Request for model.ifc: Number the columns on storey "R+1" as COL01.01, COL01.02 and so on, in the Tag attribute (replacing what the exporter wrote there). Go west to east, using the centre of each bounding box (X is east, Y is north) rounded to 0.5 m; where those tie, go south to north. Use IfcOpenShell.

First a look at what the model holds.

```python
import ifcopenshell
import ifcopenshell.util.element
import ifcopenshell.util.placement

model = ifcopenshell.open("model.ifc")
print(model.schema)
storey = next(s for s in model.by_type("IfcBuildingStorey") if s.Name == "R+1")
columns = [e for e in ifcopenshell.util.element.get_decomposition(storey) if e.is_a("IfcColumn")]
for e in sorted(columns, key=lambda e: e.id()):
    origin = ifcopenshell.util.placement.get_local_placement(e.ObjectPlacement)[:3, 3]
    print(e.id(), e.Tag, e.Name, origin.round(2) + 0.0, sep=" | ")
```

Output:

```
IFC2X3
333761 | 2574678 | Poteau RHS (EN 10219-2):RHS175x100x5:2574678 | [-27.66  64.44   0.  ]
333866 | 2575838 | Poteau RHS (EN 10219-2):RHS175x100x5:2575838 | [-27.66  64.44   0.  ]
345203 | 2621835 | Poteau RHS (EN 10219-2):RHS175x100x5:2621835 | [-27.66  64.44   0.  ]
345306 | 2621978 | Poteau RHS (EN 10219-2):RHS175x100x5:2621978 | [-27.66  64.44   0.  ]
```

```python
import ifcopenshell
import ifcopenshell.geom
import ifcopenshell.util.element
import ifcopenshell.util.shape

model = ifcopenshell.open("model.ifc")
settings = ifcopenshell.geom.settings()
settings.set("use-world-coords", True)


def centre(element):
    shape = ifcopenshell.geom.create_shape(settings, element)
    return ifcopenshell.util.shape.get_bbox_centroid(shape.geometry)


storey = next(s for s in model.by_type("IfcBuildingStorey") if s.Name == "R+1")
columns = [e for e in ifcopenshell.util.element.get_decomposition(storey) if e.is_a("IfcColumn")]

# Insertion points can sit at a corner or the storey origin, so sort by the geometry (in metres).
centres = {e: centre(e) for e in columns}
columns.sort(key=lambda e: (round(centres[e][0] / 0.5), centres[e][1]))

for i, e in enumerate(columns, start=1):
    number = f"COL01.{i:02d}"
    e.Tag = number
    print(e.id(), number)

model.write("model_rev.ifc")
```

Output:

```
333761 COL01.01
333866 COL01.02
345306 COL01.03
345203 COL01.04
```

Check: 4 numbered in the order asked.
